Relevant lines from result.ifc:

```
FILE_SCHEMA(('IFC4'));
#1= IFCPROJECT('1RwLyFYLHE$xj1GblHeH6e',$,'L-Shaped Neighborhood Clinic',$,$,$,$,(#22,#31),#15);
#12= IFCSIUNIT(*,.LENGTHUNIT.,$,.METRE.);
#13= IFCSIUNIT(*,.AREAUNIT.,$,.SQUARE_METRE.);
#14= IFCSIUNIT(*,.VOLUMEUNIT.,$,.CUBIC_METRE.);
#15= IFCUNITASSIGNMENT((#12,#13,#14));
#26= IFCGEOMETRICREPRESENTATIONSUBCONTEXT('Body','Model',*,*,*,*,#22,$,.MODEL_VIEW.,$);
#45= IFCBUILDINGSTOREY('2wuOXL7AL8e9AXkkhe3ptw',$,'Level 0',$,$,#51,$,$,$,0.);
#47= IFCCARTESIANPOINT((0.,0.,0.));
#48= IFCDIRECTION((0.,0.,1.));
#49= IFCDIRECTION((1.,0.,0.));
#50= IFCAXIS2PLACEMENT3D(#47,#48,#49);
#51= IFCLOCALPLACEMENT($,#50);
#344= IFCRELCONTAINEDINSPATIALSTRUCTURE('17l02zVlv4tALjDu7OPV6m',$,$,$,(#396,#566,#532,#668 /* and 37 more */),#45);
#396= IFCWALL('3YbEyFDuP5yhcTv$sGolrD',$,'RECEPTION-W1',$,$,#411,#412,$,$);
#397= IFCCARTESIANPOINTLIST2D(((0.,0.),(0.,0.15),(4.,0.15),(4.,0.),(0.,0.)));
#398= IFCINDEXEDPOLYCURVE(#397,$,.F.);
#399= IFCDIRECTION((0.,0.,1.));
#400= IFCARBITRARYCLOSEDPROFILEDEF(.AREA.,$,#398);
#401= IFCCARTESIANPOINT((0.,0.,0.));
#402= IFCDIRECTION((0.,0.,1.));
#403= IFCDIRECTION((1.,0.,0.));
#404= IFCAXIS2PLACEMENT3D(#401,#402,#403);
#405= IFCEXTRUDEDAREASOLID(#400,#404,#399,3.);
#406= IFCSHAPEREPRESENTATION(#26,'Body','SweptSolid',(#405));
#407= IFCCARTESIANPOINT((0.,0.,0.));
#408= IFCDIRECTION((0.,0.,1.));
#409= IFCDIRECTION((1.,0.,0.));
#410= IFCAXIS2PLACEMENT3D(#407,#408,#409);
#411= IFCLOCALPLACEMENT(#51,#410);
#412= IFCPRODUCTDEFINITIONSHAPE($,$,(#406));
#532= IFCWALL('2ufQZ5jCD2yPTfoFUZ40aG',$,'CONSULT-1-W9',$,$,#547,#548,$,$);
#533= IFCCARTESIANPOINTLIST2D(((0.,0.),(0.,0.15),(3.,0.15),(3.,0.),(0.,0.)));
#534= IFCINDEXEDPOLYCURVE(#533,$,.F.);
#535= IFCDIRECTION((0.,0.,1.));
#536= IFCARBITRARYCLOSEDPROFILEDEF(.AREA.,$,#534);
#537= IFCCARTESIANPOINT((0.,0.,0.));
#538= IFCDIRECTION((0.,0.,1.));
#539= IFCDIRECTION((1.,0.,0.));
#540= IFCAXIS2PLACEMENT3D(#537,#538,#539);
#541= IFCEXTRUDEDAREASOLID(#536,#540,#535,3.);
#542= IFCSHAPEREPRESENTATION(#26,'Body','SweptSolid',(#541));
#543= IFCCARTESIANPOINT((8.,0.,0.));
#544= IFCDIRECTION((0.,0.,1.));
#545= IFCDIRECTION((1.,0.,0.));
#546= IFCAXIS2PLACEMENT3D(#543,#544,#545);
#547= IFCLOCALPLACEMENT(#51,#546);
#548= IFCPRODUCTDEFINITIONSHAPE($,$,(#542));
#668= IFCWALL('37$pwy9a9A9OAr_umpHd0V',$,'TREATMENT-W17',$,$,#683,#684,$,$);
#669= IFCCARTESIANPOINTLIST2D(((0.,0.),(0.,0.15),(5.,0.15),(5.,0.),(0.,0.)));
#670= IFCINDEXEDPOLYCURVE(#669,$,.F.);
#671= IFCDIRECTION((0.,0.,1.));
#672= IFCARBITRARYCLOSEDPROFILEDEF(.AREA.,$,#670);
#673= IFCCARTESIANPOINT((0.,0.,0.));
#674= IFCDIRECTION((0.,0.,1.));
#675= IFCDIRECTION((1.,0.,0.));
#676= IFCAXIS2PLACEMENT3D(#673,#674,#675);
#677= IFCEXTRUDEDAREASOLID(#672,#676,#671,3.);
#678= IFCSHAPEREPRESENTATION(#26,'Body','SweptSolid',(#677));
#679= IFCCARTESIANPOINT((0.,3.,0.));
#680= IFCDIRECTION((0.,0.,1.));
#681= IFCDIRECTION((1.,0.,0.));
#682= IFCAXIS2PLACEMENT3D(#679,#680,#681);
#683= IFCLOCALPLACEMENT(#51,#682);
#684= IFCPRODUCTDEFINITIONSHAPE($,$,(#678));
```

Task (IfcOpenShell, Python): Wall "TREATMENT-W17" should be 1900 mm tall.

```python
import ifcopenshell
import ifcopenshell.geom
import ifcopenshell.util.representation
import ifcopenshell.util.shape
import ifcopenshell.util.unit

model = ifcopenshell.open("result.ifc")
unit_scale = ifcopenshell.util.unit.calculate_unit_scale(model)
settings = ifcopenshell.geom.settings()


def volume(element):
    """Net volume in cubic metres, openings subtracted."""
    shape = ifcopenshell.geom.create_shape(settings, element)
    return ifcopenshell.util.shape.get_volume(shape.geometry)


wall = model.by_guid("37$pwy9a9A9OAr_umpHd0V")
before = volume(wall)

body = ifcopenshell.util.representation.get_representation(wall, "Model", "Body")
solid = body.Items[0]
old_height = solid.Depth
solid.Depth = 1.9 / unit_scale
after = volume(wall)

print(f"height {old_height:g} -> {solid.Depth:g}, volume {before:.3f} -> {after:.3f} m3")

model.write("result_edited.ifc")
```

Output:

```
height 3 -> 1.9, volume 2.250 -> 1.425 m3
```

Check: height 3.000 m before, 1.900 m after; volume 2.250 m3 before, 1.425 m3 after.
